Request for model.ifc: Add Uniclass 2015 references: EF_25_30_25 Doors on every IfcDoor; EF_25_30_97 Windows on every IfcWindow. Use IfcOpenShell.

First a look at what the model holds.

```python
import ifcopenshell

model = ifcopenshell.open("model.ifc")
print(model.schema)
print("classifications:", [c.Name for c in model.by_type("IfcClassification")])
for ifc_class in ("IfcDoor", "IfcRoof", "IfcStair", "IfcWall", "IfcWindow"):
    print(ifc_class, len(model.by_type(ifc_class)))
```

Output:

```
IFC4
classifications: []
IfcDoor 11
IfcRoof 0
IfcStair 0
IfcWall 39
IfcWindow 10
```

```python
import ifcopenshell
import ifcopenshell.api.classification

model = ifcopenshell.open("model.ifc")

system = ifcopenshell.api.classification.add_classification(model, classification="Uniclass 2015")

codes = {
    "IfcDoor": ("EF_25_30_25", "Doors"),
    "IfcWindow": ("EF_25_30_97", "Windows"),
}
for ifc_class, (code, name) in codes.items():
    products = model.by_type(ifc_class)
    ifcopenshell.api.classification.add_reference(
        model, products=products, classification=system, identification=code, name=name
    )
    print(code, len(products))

model.write("model-out.ifc")
```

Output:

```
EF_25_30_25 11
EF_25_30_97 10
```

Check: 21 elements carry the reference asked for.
